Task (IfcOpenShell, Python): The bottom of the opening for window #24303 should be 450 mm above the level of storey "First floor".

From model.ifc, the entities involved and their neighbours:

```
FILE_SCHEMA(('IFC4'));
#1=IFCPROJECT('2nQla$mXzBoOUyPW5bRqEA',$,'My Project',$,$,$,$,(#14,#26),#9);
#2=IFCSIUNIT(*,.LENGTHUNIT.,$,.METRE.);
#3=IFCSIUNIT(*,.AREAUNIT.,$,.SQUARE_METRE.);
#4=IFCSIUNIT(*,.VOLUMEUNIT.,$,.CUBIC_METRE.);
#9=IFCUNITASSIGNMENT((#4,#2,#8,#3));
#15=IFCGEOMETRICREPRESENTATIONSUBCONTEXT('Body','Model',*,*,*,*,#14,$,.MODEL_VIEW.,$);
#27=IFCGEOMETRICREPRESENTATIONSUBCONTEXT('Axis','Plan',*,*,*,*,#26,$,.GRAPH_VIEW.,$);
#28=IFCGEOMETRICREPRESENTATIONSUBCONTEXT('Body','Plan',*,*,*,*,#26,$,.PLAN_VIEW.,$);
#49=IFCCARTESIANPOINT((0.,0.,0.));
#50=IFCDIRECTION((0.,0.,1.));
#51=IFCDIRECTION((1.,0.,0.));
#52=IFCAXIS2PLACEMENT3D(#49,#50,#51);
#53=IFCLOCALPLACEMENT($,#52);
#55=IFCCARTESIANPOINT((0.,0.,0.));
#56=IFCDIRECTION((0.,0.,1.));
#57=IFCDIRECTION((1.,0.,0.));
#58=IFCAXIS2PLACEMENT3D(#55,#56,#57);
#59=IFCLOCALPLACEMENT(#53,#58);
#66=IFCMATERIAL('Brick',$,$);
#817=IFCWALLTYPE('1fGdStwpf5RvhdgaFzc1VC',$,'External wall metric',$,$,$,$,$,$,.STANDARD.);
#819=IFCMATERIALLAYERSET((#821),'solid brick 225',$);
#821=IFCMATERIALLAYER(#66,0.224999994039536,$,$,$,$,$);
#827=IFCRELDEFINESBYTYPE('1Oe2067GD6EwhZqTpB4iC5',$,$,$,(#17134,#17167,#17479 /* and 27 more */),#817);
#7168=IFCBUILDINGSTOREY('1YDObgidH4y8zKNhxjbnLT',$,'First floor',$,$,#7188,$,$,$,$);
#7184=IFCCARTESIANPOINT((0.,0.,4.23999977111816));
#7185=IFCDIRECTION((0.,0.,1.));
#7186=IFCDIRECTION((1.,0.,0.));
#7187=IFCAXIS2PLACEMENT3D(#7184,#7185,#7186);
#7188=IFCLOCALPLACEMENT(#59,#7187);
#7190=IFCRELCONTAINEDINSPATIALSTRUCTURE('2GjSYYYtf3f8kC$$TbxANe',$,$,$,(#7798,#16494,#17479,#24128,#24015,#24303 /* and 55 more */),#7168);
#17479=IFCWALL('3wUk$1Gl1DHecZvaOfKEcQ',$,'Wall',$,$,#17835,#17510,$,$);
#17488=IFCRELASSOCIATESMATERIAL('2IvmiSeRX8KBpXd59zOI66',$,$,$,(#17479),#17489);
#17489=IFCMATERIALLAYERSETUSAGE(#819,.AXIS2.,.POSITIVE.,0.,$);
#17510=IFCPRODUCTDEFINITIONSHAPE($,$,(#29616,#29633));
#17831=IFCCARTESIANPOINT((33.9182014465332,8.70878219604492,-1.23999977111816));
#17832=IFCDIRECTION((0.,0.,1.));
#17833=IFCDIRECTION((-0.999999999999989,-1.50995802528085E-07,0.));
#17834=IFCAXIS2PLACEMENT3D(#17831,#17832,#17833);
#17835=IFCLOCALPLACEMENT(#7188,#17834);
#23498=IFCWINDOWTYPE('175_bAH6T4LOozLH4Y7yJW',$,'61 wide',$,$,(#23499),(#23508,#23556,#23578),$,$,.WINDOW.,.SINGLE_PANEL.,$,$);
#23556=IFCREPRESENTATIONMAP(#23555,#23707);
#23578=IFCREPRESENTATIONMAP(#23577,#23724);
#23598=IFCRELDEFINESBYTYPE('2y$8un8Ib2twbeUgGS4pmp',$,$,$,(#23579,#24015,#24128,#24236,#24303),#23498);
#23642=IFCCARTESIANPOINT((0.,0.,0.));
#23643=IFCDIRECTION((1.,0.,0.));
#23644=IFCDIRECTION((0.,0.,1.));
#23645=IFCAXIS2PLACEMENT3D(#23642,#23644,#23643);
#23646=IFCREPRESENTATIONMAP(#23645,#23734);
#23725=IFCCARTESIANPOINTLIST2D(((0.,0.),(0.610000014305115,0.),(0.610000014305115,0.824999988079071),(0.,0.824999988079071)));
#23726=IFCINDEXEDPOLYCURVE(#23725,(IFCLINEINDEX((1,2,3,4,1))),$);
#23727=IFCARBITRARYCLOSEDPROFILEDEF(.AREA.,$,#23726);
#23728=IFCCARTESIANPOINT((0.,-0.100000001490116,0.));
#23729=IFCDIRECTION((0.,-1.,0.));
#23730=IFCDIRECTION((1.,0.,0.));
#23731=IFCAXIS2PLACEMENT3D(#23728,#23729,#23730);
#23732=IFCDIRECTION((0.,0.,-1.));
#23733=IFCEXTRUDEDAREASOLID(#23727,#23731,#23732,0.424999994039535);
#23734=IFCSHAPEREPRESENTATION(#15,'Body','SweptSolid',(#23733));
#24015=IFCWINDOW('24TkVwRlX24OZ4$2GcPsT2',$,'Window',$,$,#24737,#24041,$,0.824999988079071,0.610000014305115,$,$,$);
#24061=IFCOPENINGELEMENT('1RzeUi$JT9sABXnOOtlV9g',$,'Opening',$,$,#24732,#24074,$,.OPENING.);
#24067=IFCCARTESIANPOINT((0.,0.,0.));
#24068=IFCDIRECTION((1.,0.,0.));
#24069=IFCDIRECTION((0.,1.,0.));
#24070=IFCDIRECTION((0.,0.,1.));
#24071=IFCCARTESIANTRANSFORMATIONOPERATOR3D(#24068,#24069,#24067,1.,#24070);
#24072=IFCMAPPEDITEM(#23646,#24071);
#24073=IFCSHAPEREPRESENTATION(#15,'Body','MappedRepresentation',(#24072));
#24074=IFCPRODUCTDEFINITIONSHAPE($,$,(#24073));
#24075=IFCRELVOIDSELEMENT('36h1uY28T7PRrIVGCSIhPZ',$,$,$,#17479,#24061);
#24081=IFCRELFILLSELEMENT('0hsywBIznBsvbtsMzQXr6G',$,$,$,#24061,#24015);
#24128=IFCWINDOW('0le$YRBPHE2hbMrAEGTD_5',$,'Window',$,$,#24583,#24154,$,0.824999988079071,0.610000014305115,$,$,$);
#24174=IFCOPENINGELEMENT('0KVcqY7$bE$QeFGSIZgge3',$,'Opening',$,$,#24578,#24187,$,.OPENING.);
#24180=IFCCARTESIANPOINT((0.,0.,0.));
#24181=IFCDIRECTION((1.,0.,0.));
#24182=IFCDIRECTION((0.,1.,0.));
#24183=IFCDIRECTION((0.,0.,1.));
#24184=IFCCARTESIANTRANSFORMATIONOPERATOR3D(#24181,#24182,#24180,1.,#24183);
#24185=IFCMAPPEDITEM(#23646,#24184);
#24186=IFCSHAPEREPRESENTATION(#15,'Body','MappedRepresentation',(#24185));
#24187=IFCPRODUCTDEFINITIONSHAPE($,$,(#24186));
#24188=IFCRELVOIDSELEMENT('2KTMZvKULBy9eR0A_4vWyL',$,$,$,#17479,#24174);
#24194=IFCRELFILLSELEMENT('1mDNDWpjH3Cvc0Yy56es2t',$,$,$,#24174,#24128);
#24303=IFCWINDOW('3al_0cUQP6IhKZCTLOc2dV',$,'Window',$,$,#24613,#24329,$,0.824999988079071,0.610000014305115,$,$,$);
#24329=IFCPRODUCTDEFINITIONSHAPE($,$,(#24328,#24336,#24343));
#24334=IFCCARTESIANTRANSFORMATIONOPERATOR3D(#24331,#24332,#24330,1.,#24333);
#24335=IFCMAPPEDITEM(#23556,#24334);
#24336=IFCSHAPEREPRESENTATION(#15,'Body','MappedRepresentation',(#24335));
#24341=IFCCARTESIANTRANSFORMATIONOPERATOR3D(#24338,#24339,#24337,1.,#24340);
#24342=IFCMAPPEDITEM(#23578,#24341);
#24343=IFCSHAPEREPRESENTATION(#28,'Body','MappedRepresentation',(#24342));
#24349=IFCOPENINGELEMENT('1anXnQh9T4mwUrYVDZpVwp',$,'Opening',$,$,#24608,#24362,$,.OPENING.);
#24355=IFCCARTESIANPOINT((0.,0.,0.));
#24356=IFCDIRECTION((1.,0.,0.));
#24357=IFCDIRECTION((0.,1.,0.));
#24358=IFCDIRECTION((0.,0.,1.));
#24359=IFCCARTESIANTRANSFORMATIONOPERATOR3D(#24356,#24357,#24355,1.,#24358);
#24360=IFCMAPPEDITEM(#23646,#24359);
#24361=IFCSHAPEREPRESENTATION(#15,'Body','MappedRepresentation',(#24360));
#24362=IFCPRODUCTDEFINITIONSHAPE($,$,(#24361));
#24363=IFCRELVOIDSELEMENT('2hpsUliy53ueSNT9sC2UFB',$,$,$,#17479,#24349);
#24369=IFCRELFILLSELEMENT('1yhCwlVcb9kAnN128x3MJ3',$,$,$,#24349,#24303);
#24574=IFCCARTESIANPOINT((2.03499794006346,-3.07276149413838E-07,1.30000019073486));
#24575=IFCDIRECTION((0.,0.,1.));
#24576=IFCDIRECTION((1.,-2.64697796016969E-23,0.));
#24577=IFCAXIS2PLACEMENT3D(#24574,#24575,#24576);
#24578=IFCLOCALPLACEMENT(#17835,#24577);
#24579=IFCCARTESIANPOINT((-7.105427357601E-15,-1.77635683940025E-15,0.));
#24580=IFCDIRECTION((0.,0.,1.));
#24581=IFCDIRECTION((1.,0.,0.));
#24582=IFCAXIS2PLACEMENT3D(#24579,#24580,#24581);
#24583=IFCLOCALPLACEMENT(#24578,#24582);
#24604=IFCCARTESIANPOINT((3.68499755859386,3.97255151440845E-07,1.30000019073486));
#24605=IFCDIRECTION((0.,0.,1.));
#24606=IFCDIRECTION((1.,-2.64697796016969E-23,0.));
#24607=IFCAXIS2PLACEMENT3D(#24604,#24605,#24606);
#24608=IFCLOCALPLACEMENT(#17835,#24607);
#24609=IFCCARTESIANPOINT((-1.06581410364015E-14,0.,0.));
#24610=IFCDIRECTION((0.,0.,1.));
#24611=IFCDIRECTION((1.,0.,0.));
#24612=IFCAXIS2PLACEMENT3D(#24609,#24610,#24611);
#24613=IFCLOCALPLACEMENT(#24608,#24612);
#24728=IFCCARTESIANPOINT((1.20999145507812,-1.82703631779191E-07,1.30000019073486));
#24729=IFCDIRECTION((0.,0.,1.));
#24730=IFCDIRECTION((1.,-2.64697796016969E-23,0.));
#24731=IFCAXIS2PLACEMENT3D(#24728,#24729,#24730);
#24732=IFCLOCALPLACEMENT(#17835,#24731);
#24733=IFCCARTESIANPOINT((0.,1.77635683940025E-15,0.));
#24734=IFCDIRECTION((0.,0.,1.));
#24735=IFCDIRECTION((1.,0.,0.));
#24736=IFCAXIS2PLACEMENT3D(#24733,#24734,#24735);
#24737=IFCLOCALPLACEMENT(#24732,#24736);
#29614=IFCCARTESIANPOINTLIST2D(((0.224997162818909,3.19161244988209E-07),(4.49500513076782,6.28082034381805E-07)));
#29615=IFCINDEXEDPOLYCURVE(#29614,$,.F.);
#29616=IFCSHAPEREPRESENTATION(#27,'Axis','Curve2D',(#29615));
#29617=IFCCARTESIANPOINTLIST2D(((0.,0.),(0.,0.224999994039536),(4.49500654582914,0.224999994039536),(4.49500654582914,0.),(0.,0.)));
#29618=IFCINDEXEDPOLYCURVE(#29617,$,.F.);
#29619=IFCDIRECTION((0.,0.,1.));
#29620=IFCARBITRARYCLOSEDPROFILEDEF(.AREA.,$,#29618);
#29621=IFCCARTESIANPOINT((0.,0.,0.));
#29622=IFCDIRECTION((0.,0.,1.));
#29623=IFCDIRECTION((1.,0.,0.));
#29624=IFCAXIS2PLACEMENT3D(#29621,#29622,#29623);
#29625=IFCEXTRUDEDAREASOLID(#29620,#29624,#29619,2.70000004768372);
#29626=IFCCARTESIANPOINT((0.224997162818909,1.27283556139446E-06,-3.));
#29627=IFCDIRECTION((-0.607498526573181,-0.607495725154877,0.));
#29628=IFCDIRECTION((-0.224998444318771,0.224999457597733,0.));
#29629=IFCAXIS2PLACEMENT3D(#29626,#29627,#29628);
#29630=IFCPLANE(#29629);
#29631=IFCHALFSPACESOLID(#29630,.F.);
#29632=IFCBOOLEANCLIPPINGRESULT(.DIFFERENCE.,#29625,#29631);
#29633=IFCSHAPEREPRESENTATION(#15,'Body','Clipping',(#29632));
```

```python
import numpy as np
import ifcopenshell
import ifcopenshell.api.geometry
import ifcopenshell.geom
import ifcopenshell.util.element
import ifcopenshell.util.placement
import ifcopenshell.util.shape
import ifcopenshell.util.unit

model = ifcopenshell.open("model.ifc")
unit_scale = ifcopenshell.util.unit.calculate_unit_scale(model)

window = model.by_id(24303)
opening = window.FillsVoids[0].RelatingOpeningElement
storey = ifcopenshell.util.element.get_container(window, ifc_class="IfcBuildingStorey")
level = ifcopenshell.util.placement.get_local_placement(storey.ObjectPlacement)[2, 3]

# The opening's origin need not be at the sill, so measure its lowest point.
shape = ifcopenshell.geom.create_shape(ifcopenshell.geom.settings(), opening)
bottom = ifcopenshell.util.shape.get_shape_bottom_elevation(shape, shape.geometry) / unit_scale
dz = level + 0.45 - bottom

shift = np.array([0.0, 0.0, dz])
# The window is placed relative to its opening, so it follows when the opening moves.
matrix = ifcopenshell.util.placement.get_local_placement(opening.ObjectPlacement)
matrix[:3, 3] += shift
ifcopenshell.api.geometry.edit_object_placement(
    model, product=opening, matrix=matrix, is_si=False, should_transform_children=True
)

print(f"moved by {dz * unit_scale:+.3f} m")

model.write("model_updated.ifc")
```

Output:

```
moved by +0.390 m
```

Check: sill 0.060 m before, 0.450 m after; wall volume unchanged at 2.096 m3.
